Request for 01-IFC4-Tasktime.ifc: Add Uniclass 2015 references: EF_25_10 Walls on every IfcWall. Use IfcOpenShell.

First a look at what the model holds.

```python
import ifcopenshell

model = ifcopenshell.open("01-IFC4-Tasktime.ifc")
print(model.schema)
print("classifications:", [c.Name for c in model.by_type("IfcClassification")])
for ifc_class in ("IfcDoor", "IfcRoof", "IfcStair", "IfcWall", "IfcWindow"):
    print(ifc_class, len(model.by_type(ifc_class)))
```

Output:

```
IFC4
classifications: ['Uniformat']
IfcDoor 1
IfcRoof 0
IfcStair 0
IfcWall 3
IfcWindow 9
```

```python
import ifcopenshell
import ifcopenshell.api.classification

model = ifcopenshell.open("01-IFC4-Tasktime.ifc")

system = ifcopenshell.api.classification.add_classification(model, classification="Uniclass 2015")

codes = {
    "IfcWall": ("EF_25_10", "Walls"),
}
for ifc_class, (code, name) in codes.items():
    products = model.by_type(ifc_class)
    ifcopenshell.api.classification.add_reference(
        model, products=products, classification=system, identification=code, name=name
    )
    print(code, len(products))

model.write("01-IFC4-Tasktime_v2.ifc")
```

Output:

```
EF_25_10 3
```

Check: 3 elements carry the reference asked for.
